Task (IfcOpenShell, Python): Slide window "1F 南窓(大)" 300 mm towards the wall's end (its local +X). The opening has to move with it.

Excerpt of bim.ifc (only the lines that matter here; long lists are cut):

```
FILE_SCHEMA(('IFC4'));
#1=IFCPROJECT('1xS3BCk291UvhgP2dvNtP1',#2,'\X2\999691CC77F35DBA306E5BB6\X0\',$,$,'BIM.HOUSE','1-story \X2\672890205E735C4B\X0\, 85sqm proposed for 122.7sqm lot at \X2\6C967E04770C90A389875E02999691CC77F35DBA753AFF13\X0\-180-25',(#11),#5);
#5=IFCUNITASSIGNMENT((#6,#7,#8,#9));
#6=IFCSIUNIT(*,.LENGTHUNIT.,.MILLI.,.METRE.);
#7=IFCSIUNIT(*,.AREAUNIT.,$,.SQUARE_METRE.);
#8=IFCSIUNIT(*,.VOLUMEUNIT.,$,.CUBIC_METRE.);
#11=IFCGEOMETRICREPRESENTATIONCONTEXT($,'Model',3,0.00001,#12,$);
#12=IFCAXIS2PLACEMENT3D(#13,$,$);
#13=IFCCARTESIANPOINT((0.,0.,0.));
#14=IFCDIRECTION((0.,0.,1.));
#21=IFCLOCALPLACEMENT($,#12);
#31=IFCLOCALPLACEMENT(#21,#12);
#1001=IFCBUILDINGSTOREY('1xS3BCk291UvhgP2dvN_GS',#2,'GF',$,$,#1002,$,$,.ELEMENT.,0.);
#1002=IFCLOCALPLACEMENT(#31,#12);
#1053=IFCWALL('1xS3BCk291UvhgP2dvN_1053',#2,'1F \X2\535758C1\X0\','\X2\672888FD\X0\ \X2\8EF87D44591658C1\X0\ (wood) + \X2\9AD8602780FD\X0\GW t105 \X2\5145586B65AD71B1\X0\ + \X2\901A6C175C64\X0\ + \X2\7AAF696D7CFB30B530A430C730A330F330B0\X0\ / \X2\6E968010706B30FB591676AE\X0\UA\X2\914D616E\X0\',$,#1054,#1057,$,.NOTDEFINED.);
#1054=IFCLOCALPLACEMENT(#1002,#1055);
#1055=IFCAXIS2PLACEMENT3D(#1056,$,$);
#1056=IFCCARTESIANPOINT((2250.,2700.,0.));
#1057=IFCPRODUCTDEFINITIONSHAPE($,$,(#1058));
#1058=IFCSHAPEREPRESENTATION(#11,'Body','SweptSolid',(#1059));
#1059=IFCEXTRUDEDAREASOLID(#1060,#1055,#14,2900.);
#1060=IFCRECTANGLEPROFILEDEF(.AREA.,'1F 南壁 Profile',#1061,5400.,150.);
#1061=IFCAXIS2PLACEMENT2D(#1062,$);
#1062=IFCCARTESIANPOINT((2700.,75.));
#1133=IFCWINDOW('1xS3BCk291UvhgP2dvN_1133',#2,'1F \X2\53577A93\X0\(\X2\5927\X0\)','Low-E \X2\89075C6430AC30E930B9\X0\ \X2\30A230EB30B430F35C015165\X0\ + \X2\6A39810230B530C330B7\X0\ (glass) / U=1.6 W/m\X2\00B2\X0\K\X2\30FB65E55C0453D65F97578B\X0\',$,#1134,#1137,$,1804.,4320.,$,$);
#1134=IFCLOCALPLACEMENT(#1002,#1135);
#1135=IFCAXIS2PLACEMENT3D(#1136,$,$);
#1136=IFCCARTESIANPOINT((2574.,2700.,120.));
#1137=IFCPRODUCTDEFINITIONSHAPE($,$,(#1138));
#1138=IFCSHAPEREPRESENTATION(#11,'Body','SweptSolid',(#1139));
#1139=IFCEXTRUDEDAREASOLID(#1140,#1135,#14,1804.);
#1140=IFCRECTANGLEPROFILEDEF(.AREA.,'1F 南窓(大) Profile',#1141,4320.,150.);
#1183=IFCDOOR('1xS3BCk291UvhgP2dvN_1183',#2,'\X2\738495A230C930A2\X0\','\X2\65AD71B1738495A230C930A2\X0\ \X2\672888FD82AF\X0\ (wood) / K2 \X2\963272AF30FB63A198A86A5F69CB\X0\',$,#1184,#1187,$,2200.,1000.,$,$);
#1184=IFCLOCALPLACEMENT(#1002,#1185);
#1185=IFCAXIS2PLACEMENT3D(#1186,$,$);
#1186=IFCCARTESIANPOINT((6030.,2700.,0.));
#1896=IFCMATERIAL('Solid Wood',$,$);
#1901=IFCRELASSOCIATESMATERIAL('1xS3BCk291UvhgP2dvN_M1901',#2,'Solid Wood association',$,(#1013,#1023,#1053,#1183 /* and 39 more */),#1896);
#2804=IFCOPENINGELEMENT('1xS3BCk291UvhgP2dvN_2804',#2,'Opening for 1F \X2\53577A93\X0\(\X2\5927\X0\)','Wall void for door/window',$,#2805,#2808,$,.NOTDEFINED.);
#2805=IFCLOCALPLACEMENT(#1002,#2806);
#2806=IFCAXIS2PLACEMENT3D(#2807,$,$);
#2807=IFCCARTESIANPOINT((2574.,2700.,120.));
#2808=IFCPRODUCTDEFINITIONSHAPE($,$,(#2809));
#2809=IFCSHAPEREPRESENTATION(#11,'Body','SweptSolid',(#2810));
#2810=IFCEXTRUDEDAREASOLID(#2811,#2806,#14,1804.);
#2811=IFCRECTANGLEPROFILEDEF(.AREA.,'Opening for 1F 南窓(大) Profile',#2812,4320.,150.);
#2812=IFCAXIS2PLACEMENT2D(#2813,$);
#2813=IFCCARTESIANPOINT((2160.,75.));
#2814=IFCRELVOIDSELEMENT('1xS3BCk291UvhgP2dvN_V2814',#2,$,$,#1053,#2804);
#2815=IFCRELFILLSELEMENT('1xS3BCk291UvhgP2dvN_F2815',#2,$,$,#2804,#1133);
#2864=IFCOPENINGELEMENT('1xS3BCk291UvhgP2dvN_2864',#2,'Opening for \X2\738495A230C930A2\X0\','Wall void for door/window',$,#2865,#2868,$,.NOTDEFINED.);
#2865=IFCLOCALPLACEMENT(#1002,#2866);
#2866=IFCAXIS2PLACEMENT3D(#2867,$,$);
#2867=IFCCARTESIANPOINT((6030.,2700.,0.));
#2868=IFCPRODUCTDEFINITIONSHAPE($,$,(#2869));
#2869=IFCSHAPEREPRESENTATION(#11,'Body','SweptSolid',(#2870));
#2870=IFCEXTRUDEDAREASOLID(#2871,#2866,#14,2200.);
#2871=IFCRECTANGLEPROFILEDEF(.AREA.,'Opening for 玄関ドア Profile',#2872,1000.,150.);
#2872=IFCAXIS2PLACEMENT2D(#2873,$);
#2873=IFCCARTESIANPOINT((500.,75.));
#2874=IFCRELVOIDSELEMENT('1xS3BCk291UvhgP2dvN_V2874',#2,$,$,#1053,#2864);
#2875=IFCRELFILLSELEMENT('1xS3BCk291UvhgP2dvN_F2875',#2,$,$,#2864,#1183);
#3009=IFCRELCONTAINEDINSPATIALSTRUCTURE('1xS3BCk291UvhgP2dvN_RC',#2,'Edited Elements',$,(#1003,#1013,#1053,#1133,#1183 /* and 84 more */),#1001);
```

```python
import ifcopenshell
import ifcopenshell.api.geometry
import ifcopenshell.util.placement

model = ifcopenshell.open("bim.ifc")

window = model.by_guid("1xS3BCk291UvhgP2dvN_1133")
opening = window.FillsVoids[0].RelatingOpeningElement
wall = opening.VoidsElements[0].RelatingBuildingElement

wall_matrix = ifcopenshell.util.placement.get_local_placement(wall.ObjectPlacement)
shift = wall_matrix[:3, 0] * 300.0
before = ifcopenshell.util.placement.get_local_placement(window.ObjectPlacement)[:3, 3].copy()

# The window is not placed relative to its opening, so move both.
for product in (opening, window):
    matrix = ifcopenshell.util.placement.get_local_placement(product.ObjectPlacement)
    matrix[:3, 3] += shift
    ifcopenshell.api.geometry.edit_object_placement(model, product=product, matrix=matrix, is_si=False)

after = ifcopenshell.util.placement.get_local_placement(window.ObjectPlacement)[:3, 3]
print("window moved by", (after - before).round(3) + 0.0)

model.write("bim_v2.ifc")
```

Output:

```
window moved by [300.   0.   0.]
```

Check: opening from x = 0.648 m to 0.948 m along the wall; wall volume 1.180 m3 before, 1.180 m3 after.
